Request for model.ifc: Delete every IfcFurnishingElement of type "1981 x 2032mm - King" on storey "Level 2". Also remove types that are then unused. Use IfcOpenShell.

First a look at what the model holds.

```python
import ifcopenshell
import ifcopenshell.util.element

model = ifcopenshell.open("model.ifc")
print(model.schema)
storey = next(s for s in model.by_type("IfcBuildingStorey") if s.Name == "Level 2")
furniture = [e for e in ifcopenshell.util.element.get_decomposition(storey) if e.is_a("IfcFurnishingElement")]
seen = {}
for e in furniture:
    element_type = ifcopenshell.util.element.get_type(e)
    name = element_type.Name if element_type not in (None, e) else None
    seen[name] = seen.get(name, 0) + 1
for name, count in sorted(seen.items(), key=str):
    print(count, "x", name)
```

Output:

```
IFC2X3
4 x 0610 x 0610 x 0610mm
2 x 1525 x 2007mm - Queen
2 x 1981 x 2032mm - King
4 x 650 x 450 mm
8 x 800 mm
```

```python
import ifcopenshell
import ifcopenshell.api.root
import ifcopenshell.util.element

model = ifcopenshell.open("model.ifc")

storey = next(s for s in model.by_type("IfcBuildingStorey") if s.Name == "Level 2")
furniture = [e for e in ifcopenshell.util.element.get_decomposition(storey) if e.is_a("IfcFurnishingElement")]
targets = [e for e in furniture if (t := ifcopenshell.util.element.get_type(e)) not in (None, e) and t.Name == "1981 x 2032mm - King"]
types = {ifcopenshell.util.element.get_type(e) for e in targets} - {None, *targets}

for e in targets:
    ifcopenshell.api.root.remove_product(model, product=e)
print(len(targets), "removed")

unused = [t for t in types if not ifcopenshell.util.element.get_types(t)]
for t in unused:
    ifcopenshell.api.root.remove_product(model, product=t)
print(len(unused), "unused types removed")

model.write("model_edited.ifc")
```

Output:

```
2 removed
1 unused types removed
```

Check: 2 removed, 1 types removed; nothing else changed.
